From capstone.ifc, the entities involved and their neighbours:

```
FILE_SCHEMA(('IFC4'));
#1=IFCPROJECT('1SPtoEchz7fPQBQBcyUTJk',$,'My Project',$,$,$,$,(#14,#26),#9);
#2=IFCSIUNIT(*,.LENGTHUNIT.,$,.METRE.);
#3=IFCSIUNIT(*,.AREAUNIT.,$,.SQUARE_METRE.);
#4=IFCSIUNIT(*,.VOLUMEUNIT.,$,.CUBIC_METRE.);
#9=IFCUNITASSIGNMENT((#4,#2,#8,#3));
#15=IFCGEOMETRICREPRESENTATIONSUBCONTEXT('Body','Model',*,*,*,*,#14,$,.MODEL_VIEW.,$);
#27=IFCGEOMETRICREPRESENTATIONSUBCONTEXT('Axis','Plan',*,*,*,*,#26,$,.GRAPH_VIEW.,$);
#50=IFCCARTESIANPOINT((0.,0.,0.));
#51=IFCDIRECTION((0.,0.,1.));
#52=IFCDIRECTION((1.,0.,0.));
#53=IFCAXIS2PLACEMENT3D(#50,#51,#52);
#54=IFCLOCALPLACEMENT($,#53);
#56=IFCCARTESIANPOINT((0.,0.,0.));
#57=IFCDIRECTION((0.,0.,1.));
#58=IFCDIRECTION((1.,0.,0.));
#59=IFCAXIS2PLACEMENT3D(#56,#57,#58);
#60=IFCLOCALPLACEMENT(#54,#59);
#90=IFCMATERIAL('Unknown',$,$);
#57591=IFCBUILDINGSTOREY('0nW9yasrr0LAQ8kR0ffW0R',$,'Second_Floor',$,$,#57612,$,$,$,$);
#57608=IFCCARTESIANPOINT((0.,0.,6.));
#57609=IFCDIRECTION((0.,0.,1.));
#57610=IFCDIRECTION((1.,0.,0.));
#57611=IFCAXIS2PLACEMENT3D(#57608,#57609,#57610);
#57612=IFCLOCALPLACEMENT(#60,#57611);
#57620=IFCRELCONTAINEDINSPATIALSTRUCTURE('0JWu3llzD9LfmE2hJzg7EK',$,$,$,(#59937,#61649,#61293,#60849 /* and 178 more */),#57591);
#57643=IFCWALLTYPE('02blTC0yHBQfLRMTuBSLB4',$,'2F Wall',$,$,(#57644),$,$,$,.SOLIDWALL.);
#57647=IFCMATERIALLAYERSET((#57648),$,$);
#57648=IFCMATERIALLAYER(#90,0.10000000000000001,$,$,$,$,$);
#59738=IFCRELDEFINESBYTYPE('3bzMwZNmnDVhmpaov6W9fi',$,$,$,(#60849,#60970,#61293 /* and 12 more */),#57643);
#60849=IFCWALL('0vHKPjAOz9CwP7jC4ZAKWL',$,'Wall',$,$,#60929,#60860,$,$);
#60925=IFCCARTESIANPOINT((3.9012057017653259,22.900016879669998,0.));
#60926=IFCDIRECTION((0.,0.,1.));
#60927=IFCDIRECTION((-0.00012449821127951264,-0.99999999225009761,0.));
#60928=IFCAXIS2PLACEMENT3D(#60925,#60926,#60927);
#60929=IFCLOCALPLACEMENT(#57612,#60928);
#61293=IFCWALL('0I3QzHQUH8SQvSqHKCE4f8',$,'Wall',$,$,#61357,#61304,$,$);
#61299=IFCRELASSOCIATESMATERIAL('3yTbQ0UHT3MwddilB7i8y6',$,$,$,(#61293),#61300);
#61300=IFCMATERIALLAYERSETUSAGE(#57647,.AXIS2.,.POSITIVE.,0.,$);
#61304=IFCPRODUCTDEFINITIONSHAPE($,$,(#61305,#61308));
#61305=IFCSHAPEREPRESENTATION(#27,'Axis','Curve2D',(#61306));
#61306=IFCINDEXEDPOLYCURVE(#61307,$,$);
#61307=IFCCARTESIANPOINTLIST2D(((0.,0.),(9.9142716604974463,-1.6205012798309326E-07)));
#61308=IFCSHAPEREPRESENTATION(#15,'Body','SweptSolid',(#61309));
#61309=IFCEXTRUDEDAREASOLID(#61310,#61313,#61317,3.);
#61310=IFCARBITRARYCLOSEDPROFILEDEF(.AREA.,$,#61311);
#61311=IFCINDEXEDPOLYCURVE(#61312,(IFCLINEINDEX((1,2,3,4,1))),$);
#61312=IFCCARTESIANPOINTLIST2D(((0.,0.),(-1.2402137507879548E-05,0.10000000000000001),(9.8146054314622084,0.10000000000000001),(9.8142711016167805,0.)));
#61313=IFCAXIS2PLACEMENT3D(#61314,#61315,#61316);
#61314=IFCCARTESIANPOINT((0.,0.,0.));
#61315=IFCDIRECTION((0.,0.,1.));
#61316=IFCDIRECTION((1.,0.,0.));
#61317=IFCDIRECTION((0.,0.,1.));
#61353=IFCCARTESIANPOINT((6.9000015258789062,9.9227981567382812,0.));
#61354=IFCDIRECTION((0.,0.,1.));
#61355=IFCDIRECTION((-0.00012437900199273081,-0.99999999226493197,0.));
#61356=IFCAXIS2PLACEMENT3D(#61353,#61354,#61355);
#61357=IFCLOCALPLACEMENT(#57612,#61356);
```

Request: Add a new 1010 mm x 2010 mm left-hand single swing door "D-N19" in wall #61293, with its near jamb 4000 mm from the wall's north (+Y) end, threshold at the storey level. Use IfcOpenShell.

```python
import numpy as np
import ifcopenshell
import ifcopenshell.api.feature
import ifcopenshell.api.geometry
import ifcopenshell.api.root
import ifcopenshell.api.spatial
import ifcopenshell.geom
import ifcopenshell.util.element
import ifcopenshell.util.placement
import ifcopenshell.util.representation
import ifcopenshell.util.shape
import ifcopenshell.util.unit

model = ifcopenshell.open("capstone.ifc")
unit_scale = ifcopenshell.util.unit.calculate_unit_scale(model)
settings = ifcopenshell.geom.settings()


def volume(element):
    """Net volume in cubic metres, openings subtracted."""
    shape = ifcopenshell.geom.create_shape(settings, element)
    return ifcopenshell.util.shape.get_volume(shape.geometry)


wall = model.by_id(61293)
storey = ifcopenshell.util.element.get_container(wall, ifc_class="IfcBuildingStorey")
context = ifcopenshell.util.representation.get_context(model, "Model", "Body", "MODEL_VIEW")
before = volume(wall)

width, height, from_end, sill = 1.01, 2.01, 4, 0.0  # metres

# The wall runs along its own X axis, and the end named is its -X end.
wall_shape = ifcopenshell.geom.create_shape(settings, wall)
x, y, z = ifcopenshell.util.shape.get_vertices(wall_shape.geometry).T
start = x.min() + from_end
face, thickness = float(y.min()), float(y.max() - y.min())
wall_matrix = ifcopenshell.util.placement.get_local_placement(wall.ObjectPlacement)
level = ifcopenshell.util.placement.get_local_placement(storey.ObjectPlacement)[2, 3]


def in_wall(x, y):
    """Placement at x, y metres in the wall's axes, at sill height."""
    matrix = wall_matrix.copy()
    matrix[:, 3] = wall_matrix @ np.array([x / unit_scale, y / unit_scale, 0.0, 1.0])
    matrix[2, 3] = level + sill / unit_scale
    return matrix


# Opening: a box that overshoots both wall faces by 50 mm.
opening = ifcopenshell.api.root.create_entity(model, ifc_class="IfcOpeningElement", predefined_type="OPENING")
box = ifcopenshell.api.geometry.add_wall_representation(
    model, context=context, length=width, height=height, thickness=thickness + 0.1
)
ifcopenshell.api.geometry.assign_representation(model, product=opening, representation=box)
ifcopenshell.api.geometry.edit_object_placement(model, product=opening, matrix=in_wall(start, face - 0.05), is_si=False)
ifcopenshell.api.feature.add_feature(model, feature=opening, element=wall)

door = ifcopenshell.api.root.create_entity(model, ifc_class="IfcDoor", name="D-N19", predefined_type="DOOR")
door.OverallWidth, door.OverallHeight = width / unit_scale, height / unit_scale
door.OperationType = "SINGLE_SWING_LEFT"
body = ifcopenshell.api.geometry.add_door_representation(
    model,
    context=context,
    overall_width=door.OverallWidth,
    overall_height=door.OverallHeight,
    operation_type="SINGLE_SWING_LEFT",
    lining_properties={"LiningDepth": thickness / unit_scale, "ThresholdDepth": thickness / unit_scale},
)
ifcopenshell.api.geometry.assign_representation(model, product=door, representation=body)
ifcopenshell.api.spatial.assign_container(model, products=[door], relating_structure=storey)
ifcopenshell.api.feature.add_filling(model, opening=opening, element=door)

# The lining spans the wall, so the door starts at the wall face.
ifcopenshell.api.geometry.edit_object_placement(model, product=door, matrix=in_wall(start, face), is_si=False)

after = volume(wall)

print(f"wall volume {before:.3f} -> {after:.3f} m3")

model.write("capstone_edited.ifc")
```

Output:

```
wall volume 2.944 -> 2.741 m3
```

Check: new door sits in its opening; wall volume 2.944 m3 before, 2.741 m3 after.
